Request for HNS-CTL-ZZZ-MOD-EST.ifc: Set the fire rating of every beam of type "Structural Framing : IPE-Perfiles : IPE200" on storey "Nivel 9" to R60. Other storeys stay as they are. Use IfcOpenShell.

First a look at what the model holds.

```python
import ifcopenshell
import ifcopenshell.util.element

model = ifcopenshell.open("HNS-CTL-ZZZ-MOD-EST.ifc")
print(model.schema)
storey = next(s for s in model.by_type("IfcBuildingStorey") if s.Name == "Nivel 9")
beams = [e for e in ifcopenshell.util.element.get_decomposition(storey) if e.is_a("IfcBeam")]
seen = {}
for e in beams:
    element_type = ifcopenshell.util.element.get_type(e)
    key = (element_type.Name if element_type != e and element_type else None, ifcopenshell.util.element.get_pset(e, "Pset_BeamCommon", "FireRating"))
    seen[key] = seen.get(key, 0) + 1
for (name, value), count in sorted(seen.items(), key=str):
    print(count, "x", name, "|", value)
```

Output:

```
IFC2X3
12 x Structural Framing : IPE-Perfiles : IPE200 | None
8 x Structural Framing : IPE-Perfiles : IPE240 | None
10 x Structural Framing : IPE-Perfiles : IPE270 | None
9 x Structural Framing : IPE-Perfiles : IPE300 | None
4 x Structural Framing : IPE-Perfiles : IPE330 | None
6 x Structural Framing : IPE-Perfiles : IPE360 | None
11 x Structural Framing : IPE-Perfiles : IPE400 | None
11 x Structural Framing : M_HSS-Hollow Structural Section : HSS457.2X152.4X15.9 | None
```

```python
import ifcopenshell
import ifcopenshell.api.pset
import ifcopenshell.util.element

model = ifcopenshell.open("HNS-CTL-ZZZ-MOD-EST.ifc")

storey = next(s for s in model.by_type("IfcBuildingStorey") if s.Name == "Nivel 9")
beams = [e for e in ifcopenshell.util.element.get_decomposition(storey) if e.is_a("IfcBeam")]

count = 0
for e in beams:
    element_type = ifcopenshell.util.element.get_type(e)
    if element_type in (None, e) or element_type.Name != "Structural Framing : IPE-Perfiles : IPE200":
        continue
    # add_pset returns the element's existing set when there is one.
    pset = ifcopenshell.api.pset.add_pset(model, product=e, name="Pset_BeamCommon")
    ifcopenshell.api.pset.edit_pset(model, pset=pset, properties={"FireRating": "R60"})
    count += 1

print(count, "beams updated")

model.write("HNS-CTL-ZZZ-MOD-EST-out.ifc")
```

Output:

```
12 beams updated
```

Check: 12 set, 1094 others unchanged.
